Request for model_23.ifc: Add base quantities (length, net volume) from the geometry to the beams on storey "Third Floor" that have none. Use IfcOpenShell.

First a look at what the model holds.

```python
import ifcopenshell
import ifcopenshell.util.element
import ifcopenshell.util.unit

model = ifcopenshell.open("model_23.ifc")
print(model.schema)
for unit_type in ("LENGTHUNIT", "AREAUNIT", "VOLUMEUNIT"):
    print(unit_type, ifcopenshell.util.unit.calculate_unit_scale(model, unit_type))
storey = next(s for s in model.by_type("IfcBuildingStorey") if s.Name == "Third Floor")
beams = [e for e in ifcopenshell.util.element.get_decomposition(storey) if e.is_a("IfcBeam")]
for e in sorted(beams, key=lambda e: e.id()):
    print(e.id(), e.is_a(), e.Name, list(ifcopenshell.util.element.get_psets(e, qtos_only=True)), sep=" | ")
```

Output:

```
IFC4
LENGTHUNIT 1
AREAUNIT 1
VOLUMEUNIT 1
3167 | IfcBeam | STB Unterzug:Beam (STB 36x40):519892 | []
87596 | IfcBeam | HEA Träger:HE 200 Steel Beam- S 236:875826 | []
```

```python
import ifcopenshell
import ifcopenshell.api.pset
import ifcopenshell.geom
import ifcopenshell.util.element
import ifcopenshell.util.shape
import ifcopenshell.util.unit

model = ifcopenshell.open("model_23.ifc")
unit_scale = ifcopenshell.util.unit.calculate_unit_scale(model)
volume_scale = ifcopenshell.util.unit.calculate_unit_scale(model, "VOLUMEUNIT")
settings = ifcopenshell.geom.settings()

storey = next(s for s in model.by_type("IfcBuildingStorey") if s.Name == "Third Floor")
beams = [e for e in ifcopenshell.util.element.get_decomposition(storey) if e.is_a("IfcBeam")]

for e in sorted(beams, key=lambda e: e.id()):
    if ifcopenshell.util.element.get_psets(e, qtos_only=True, should_inherit=False):
        continue
    # Geometry comes back in metres, in the element's own axes.
    shape = ifcopenshell.geom.create_shape(settings, e)
    values = {
        "Length": ifcopenshell.util.shape.get_max_xyz(shape.geometry) / unit_scale,
        "NetVolume": ifcopenshell.util.shape.get_volume(shape.geometry) / volume_scale,
    }
    qto = ifcopenshell.api.pset.add_qto(model, product=e, name="Qto_BeamBaseQuantities")
    ifcopenshell.api.pset.edit_qto(model, qto=qto, properties=values)
    print(e.id(), {k: round(v, 3) for k, v in values.items()})

model.write("model_23_edited.ifc")
```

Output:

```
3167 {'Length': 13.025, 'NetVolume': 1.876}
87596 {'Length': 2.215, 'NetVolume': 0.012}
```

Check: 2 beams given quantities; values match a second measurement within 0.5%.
